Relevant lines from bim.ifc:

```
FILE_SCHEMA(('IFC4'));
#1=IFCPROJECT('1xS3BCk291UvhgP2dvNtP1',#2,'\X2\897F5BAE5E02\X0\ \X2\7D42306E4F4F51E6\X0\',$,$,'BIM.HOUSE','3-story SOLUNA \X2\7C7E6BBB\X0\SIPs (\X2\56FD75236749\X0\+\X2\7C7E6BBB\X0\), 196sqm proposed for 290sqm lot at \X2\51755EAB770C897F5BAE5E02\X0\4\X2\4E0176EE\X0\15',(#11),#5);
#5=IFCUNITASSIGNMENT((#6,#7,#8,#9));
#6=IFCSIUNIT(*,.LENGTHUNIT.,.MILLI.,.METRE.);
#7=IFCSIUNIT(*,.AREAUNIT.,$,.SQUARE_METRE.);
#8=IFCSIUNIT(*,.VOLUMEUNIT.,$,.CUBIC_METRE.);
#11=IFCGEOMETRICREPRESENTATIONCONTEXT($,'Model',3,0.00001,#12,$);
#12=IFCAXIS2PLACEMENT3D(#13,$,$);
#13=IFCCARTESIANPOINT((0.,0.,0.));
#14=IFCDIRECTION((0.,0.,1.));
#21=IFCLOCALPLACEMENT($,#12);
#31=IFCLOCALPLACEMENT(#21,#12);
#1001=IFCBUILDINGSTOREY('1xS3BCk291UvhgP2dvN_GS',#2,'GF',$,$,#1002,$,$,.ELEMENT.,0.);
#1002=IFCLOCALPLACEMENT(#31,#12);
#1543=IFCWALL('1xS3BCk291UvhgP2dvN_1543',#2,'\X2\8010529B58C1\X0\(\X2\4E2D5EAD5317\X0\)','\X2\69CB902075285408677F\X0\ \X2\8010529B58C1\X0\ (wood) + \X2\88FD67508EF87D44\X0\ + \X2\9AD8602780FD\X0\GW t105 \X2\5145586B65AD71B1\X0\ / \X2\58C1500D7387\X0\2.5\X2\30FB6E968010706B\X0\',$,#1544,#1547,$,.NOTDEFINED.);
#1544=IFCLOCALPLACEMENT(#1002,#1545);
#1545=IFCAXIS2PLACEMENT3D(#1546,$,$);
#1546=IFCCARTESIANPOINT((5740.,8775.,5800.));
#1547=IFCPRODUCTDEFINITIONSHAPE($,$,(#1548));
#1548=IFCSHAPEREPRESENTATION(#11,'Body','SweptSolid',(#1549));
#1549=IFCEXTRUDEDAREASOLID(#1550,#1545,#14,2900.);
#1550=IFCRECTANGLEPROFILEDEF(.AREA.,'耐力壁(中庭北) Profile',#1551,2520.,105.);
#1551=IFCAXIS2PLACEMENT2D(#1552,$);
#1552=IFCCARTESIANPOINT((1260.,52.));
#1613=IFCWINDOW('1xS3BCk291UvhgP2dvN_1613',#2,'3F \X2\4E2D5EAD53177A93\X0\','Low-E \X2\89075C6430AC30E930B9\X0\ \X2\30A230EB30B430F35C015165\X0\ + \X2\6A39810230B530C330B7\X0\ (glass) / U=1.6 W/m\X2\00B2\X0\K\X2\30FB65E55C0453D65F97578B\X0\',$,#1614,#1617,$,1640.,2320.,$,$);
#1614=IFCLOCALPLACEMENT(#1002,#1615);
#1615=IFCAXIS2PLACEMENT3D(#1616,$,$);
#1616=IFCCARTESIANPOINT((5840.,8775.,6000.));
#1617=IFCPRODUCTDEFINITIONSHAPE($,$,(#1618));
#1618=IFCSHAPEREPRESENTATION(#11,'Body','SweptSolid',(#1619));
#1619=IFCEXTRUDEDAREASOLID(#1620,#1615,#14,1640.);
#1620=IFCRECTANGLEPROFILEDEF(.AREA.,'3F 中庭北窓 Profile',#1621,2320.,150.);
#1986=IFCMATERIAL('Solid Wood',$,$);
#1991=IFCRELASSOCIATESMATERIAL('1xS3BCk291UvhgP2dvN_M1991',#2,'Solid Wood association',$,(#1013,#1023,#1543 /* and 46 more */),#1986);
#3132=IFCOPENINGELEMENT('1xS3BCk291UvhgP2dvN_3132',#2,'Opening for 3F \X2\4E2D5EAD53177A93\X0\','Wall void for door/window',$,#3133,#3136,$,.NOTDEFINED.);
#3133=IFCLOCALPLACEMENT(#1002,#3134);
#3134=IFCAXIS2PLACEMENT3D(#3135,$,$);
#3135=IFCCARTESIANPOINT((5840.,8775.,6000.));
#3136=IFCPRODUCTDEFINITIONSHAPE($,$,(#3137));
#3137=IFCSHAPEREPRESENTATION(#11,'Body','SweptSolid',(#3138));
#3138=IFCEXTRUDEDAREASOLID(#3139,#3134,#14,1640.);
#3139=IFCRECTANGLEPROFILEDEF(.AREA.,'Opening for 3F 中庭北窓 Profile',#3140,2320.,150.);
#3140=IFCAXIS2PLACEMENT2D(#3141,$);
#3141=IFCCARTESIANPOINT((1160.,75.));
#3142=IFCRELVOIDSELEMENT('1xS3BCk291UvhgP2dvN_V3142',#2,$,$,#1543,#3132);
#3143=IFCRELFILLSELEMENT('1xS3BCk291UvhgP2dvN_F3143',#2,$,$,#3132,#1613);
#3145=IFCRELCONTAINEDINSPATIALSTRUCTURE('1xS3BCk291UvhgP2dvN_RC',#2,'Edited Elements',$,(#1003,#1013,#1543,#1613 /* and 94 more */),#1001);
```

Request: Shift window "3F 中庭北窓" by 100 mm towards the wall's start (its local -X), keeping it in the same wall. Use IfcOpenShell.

```python
import ifcopenshell
import ifcopenshell.api.geometry
import ifcopenshell.util.placement
import ifcopenshell.util.unit

model = ifcopenshell.open("bim.ifc")
unit_scale = ifcopenshell.util.unit.calculate_unit_scale(model)

window = model.by_id(1613)
opening = window.FillsVoids[0].RelatingOpeningElement
wall = opening.VoidsElements[0].RelatingBuildingElement

wall_matrix = ifcopenshell.util.placement.get_local_placement(wall.ObjectPlacement)
shift = wall_matrix[:3, 0] * -0.1 / unit_scale
before = ifcopenshell.util.placement.get_local_placement(window.ObjectPlacement)[:3, 3].copy()

# The window is not placed relative to its opening, so move both.
for product in (opening, window):
    matrix = ifcopenshell.util.placement.get_local_placement(product.ObjectPlacement)
    matrix[:3, 3] += shift
    ifcopenshell.api.geometry.edit_object_placement(model, product=product, matrix=matrix, is_si=False)

after = ifcopenshell.util.placement.get_local_placement(window.ObjectPlacement)[:3, 3]
print("window moved by", (after - before).round(3) + 0.0)

model.write("bim_edited.ifc")
```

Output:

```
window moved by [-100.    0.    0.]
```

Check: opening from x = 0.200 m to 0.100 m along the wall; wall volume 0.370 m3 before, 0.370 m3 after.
